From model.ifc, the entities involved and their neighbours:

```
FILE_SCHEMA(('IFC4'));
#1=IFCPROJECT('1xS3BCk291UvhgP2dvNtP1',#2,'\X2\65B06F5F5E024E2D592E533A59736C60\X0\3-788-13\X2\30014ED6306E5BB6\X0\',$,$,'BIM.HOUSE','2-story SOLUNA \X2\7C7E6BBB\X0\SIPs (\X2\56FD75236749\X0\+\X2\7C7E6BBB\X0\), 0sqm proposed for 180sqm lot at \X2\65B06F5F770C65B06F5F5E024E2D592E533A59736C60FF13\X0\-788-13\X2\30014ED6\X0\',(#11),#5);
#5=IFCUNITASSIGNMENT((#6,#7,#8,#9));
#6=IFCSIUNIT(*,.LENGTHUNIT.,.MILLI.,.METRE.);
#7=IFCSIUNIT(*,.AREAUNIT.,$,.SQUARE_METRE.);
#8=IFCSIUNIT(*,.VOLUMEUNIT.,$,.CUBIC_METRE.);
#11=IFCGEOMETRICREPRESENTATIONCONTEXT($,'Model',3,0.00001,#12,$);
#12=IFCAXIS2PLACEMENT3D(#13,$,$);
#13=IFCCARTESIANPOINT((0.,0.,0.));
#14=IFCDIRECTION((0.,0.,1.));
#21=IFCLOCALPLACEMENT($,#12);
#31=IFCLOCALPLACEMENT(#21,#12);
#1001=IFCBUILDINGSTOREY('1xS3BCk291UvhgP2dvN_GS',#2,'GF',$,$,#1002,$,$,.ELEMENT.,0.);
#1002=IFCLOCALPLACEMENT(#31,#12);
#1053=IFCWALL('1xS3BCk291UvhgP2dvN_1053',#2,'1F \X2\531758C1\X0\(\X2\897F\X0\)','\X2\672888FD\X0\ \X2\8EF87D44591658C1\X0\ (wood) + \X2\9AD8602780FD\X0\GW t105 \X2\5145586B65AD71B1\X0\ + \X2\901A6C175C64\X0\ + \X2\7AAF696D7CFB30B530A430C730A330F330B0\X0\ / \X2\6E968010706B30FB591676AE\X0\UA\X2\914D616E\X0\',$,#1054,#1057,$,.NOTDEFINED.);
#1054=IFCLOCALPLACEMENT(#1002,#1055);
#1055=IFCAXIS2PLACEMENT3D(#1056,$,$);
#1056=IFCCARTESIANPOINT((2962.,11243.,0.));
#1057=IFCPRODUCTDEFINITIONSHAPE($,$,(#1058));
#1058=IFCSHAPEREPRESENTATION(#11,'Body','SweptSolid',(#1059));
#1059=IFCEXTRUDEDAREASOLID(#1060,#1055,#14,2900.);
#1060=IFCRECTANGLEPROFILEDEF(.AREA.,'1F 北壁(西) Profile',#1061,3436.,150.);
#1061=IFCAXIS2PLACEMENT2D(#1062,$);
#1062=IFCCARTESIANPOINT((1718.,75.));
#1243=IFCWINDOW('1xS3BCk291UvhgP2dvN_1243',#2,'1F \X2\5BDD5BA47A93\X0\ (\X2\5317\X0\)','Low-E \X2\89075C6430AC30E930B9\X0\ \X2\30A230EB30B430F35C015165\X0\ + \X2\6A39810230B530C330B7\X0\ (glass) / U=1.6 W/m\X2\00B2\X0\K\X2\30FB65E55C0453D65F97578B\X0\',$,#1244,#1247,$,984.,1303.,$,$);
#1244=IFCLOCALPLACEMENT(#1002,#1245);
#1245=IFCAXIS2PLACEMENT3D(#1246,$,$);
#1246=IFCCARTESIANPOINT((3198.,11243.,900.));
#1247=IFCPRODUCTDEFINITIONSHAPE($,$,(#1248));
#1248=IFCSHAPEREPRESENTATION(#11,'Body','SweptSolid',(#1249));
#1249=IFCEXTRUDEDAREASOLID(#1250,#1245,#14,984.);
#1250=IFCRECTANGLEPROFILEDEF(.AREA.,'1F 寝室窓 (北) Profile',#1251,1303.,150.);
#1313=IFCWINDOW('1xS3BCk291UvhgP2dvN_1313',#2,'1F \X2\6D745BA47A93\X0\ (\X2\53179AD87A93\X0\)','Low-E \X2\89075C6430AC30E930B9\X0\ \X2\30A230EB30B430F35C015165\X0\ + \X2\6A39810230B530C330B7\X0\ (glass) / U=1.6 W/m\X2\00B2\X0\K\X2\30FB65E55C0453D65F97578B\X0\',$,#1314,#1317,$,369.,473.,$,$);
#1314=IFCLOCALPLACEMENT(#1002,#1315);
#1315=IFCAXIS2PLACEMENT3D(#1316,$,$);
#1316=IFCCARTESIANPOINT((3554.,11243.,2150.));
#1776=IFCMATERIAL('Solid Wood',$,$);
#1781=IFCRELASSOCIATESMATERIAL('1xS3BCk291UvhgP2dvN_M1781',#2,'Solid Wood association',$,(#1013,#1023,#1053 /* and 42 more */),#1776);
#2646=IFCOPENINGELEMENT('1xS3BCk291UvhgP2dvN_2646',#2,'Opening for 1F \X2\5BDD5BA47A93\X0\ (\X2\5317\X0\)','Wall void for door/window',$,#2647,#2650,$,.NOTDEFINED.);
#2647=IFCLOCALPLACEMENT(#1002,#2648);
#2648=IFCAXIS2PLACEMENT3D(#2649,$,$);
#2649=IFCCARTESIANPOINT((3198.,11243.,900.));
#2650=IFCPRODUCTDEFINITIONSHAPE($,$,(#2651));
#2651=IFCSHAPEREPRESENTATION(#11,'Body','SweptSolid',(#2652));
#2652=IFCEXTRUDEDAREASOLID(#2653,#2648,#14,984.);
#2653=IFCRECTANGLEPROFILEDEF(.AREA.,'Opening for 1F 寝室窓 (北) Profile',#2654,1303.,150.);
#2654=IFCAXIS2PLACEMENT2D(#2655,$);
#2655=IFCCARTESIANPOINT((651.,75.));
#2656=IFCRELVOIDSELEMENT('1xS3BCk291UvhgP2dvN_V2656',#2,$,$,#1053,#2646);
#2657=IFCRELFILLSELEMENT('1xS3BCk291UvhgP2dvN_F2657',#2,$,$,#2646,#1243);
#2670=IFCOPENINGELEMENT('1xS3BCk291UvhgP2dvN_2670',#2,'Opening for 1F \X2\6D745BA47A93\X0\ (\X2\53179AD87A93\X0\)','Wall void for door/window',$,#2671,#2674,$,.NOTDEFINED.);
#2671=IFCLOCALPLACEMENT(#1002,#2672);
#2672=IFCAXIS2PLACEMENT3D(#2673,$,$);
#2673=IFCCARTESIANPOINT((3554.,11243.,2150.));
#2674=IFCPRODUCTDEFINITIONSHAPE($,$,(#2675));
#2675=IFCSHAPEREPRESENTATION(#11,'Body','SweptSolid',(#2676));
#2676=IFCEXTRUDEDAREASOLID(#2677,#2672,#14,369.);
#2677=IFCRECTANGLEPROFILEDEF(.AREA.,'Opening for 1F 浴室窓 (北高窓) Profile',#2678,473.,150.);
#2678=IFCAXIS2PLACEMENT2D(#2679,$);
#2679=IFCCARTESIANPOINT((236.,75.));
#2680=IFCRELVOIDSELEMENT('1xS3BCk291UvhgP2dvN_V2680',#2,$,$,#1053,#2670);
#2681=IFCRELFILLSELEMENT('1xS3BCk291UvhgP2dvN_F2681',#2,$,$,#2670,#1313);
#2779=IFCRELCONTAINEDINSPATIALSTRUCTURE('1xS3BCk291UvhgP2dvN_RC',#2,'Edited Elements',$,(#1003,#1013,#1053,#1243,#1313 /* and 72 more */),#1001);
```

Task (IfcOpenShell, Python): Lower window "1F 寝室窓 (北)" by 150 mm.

```python
import numpy as np
import ifcopenshell
import ifcopenshell.api.geometry
import ifcopenshell.util.placement
import ifcopenshell.util.unit

model = ifcopenshell.open("model.ifc")
unit_scale = ifcopenshell.util.unit.calculate_unit_scale(model)

window = model.by_id(1243)
opening = window.FillsVoids[0].RelatingOpeningElement
dz = -0.15 / unit_scale

shift = np.array([0.0, 0.0, dz])
# The window is not placed relative to its opening, so move both.
for product in (opening, window):
    matrix = ifcopenshell.util.placement.get_local_placement(product.ObjectPlacement)
    matrix[:3, 3] += shift
    ifcopenshell.api.geometry.edit_object_placement(model, product=product, matrix=matrix, is_si=False)

print(f"moved by {dz * unit_scale:+.3f} m")

model.write("model_v2.ifc")
```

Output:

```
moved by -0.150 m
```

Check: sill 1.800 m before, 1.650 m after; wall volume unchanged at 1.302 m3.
